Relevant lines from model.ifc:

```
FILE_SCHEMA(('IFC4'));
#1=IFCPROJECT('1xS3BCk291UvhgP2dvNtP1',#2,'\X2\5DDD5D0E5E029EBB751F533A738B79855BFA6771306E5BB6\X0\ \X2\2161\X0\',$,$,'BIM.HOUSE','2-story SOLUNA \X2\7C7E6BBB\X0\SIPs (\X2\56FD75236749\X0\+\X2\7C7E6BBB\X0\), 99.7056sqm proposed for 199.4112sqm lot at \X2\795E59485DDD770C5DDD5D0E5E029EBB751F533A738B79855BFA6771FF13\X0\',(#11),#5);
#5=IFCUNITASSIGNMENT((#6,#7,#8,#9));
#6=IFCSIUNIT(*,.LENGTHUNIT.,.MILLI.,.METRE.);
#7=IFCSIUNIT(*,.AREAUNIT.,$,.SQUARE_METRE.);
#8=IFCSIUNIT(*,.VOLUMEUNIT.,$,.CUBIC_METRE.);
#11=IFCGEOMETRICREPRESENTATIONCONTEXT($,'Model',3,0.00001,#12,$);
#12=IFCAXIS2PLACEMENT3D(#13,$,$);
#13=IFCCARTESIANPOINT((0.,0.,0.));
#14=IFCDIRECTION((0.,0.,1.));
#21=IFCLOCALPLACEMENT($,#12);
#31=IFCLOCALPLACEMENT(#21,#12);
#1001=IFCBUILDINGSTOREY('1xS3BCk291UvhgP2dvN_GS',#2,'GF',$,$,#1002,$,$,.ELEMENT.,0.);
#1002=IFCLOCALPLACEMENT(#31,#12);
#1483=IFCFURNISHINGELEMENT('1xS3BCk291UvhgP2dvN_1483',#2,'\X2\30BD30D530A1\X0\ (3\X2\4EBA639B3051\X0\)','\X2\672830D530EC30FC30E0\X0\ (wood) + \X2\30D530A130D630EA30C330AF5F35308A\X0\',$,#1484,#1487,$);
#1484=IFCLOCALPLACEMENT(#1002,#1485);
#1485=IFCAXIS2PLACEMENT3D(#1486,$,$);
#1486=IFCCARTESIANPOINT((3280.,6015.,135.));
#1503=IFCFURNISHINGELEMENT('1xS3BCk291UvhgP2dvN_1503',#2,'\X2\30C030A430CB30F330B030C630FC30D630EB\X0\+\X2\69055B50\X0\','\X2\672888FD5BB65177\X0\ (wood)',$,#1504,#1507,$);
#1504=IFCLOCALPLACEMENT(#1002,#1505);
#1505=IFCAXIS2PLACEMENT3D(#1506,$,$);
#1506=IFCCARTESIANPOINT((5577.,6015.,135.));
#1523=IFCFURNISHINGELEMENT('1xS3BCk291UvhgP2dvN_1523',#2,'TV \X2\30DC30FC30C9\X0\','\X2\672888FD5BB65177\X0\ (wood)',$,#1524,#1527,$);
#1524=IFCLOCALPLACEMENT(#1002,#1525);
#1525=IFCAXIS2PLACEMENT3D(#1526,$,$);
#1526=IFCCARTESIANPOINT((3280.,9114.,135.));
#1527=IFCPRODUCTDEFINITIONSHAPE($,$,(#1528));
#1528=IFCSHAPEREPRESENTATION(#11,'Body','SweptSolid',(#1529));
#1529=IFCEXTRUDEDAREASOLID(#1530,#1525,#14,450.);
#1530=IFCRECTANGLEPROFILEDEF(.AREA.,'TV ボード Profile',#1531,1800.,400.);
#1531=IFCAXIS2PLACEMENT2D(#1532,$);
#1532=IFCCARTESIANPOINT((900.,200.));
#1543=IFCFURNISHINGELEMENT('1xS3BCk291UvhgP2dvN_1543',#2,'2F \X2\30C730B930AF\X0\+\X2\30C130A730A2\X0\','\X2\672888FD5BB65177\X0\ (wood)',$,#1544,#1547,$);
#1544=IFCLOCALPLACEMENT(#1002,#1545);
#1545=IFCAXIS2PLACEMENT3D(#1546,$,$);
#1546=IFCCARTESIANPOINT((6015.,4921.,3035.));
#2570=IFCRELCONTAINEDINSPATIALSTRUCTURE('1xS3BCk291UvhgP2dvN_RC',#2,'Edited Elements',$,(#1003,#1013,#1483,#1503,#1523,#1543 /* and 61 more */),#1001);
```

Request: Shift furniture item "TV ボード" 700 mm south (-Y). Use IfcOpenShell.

```python
import ifcopenshell
import ifcopenshell.api.geometry
import ifcopenshell.util.placement

model = ifcopenshell.open("model.ifc")

item = model.by_guid("1xS3BCk291UvhgP2dvN_1523")
matrix = ifcopenshell.util.placement.get_local_placement(item.ObjectPlacement)
matrix[1, 3] -= 700.0
ifcopenshell.api.geometry.edit_object_placement(model, product=item, matrix=matrix, is_si=False)

print(ifcopenshell.util.placement.get_local_placement(item.ObjectPlacement).round(3) + 0.0)

model.write("model_edited.ifc")
```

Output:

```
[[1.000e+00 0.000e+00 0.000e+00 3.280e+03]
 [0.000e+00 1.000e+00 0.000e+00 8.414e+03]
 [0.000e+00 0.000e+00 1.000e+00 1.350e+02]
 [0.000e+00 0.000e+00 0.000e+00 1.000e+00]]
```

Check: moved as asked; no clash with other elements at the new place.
